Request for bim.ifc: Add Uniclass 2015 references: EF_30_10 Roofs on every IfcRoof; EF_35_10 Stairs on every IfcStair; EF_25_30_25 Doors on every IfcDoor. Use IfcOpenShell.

First a look at what the model holds.

```python
import ifcopenshell

model = ifcopenshell.open("bim.ifc")
print(model.schema)
print("classifications:", [c.Name for c in model.by_type("IfcClassification")])
for ifc_class in ("IfcDoor", "IfcRoof", "IfcStair", "IfcWall", "IfcWindow"):
    print(ifc_class, len(model.by_type(ifc_class)))
```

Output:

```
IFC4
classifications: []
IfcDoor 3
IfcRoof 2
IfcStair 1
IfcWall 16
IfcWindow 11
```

```python
import ifcopenshell
import ifcopenshell.api.classification

model = ifcopenshell.open("bim.ifc")

system = ifcopenshell.api.classification.add_classification(model, classification="Uniclass 2015")

codes = {
    "IfcRoof": ("EF_30_10", "Roofs"),
    "IfcStair": ("EF_35_10", "Stairs"),
    "IfcDoor": ("EF_25_30_25", "Doors"),
}
for ifc_class, (code, name) in codes.items():
    products = model.by_type(ifc_class)
    ifcopenshell.api.classification.add_reference(
        model, products=products, classification=system, identification=code, name=name
    )
    print(code, len(products))

model.write("bim_v2.ifc")
```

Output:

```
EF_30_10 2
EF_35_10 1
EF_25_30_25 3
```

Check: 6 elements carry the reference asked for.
